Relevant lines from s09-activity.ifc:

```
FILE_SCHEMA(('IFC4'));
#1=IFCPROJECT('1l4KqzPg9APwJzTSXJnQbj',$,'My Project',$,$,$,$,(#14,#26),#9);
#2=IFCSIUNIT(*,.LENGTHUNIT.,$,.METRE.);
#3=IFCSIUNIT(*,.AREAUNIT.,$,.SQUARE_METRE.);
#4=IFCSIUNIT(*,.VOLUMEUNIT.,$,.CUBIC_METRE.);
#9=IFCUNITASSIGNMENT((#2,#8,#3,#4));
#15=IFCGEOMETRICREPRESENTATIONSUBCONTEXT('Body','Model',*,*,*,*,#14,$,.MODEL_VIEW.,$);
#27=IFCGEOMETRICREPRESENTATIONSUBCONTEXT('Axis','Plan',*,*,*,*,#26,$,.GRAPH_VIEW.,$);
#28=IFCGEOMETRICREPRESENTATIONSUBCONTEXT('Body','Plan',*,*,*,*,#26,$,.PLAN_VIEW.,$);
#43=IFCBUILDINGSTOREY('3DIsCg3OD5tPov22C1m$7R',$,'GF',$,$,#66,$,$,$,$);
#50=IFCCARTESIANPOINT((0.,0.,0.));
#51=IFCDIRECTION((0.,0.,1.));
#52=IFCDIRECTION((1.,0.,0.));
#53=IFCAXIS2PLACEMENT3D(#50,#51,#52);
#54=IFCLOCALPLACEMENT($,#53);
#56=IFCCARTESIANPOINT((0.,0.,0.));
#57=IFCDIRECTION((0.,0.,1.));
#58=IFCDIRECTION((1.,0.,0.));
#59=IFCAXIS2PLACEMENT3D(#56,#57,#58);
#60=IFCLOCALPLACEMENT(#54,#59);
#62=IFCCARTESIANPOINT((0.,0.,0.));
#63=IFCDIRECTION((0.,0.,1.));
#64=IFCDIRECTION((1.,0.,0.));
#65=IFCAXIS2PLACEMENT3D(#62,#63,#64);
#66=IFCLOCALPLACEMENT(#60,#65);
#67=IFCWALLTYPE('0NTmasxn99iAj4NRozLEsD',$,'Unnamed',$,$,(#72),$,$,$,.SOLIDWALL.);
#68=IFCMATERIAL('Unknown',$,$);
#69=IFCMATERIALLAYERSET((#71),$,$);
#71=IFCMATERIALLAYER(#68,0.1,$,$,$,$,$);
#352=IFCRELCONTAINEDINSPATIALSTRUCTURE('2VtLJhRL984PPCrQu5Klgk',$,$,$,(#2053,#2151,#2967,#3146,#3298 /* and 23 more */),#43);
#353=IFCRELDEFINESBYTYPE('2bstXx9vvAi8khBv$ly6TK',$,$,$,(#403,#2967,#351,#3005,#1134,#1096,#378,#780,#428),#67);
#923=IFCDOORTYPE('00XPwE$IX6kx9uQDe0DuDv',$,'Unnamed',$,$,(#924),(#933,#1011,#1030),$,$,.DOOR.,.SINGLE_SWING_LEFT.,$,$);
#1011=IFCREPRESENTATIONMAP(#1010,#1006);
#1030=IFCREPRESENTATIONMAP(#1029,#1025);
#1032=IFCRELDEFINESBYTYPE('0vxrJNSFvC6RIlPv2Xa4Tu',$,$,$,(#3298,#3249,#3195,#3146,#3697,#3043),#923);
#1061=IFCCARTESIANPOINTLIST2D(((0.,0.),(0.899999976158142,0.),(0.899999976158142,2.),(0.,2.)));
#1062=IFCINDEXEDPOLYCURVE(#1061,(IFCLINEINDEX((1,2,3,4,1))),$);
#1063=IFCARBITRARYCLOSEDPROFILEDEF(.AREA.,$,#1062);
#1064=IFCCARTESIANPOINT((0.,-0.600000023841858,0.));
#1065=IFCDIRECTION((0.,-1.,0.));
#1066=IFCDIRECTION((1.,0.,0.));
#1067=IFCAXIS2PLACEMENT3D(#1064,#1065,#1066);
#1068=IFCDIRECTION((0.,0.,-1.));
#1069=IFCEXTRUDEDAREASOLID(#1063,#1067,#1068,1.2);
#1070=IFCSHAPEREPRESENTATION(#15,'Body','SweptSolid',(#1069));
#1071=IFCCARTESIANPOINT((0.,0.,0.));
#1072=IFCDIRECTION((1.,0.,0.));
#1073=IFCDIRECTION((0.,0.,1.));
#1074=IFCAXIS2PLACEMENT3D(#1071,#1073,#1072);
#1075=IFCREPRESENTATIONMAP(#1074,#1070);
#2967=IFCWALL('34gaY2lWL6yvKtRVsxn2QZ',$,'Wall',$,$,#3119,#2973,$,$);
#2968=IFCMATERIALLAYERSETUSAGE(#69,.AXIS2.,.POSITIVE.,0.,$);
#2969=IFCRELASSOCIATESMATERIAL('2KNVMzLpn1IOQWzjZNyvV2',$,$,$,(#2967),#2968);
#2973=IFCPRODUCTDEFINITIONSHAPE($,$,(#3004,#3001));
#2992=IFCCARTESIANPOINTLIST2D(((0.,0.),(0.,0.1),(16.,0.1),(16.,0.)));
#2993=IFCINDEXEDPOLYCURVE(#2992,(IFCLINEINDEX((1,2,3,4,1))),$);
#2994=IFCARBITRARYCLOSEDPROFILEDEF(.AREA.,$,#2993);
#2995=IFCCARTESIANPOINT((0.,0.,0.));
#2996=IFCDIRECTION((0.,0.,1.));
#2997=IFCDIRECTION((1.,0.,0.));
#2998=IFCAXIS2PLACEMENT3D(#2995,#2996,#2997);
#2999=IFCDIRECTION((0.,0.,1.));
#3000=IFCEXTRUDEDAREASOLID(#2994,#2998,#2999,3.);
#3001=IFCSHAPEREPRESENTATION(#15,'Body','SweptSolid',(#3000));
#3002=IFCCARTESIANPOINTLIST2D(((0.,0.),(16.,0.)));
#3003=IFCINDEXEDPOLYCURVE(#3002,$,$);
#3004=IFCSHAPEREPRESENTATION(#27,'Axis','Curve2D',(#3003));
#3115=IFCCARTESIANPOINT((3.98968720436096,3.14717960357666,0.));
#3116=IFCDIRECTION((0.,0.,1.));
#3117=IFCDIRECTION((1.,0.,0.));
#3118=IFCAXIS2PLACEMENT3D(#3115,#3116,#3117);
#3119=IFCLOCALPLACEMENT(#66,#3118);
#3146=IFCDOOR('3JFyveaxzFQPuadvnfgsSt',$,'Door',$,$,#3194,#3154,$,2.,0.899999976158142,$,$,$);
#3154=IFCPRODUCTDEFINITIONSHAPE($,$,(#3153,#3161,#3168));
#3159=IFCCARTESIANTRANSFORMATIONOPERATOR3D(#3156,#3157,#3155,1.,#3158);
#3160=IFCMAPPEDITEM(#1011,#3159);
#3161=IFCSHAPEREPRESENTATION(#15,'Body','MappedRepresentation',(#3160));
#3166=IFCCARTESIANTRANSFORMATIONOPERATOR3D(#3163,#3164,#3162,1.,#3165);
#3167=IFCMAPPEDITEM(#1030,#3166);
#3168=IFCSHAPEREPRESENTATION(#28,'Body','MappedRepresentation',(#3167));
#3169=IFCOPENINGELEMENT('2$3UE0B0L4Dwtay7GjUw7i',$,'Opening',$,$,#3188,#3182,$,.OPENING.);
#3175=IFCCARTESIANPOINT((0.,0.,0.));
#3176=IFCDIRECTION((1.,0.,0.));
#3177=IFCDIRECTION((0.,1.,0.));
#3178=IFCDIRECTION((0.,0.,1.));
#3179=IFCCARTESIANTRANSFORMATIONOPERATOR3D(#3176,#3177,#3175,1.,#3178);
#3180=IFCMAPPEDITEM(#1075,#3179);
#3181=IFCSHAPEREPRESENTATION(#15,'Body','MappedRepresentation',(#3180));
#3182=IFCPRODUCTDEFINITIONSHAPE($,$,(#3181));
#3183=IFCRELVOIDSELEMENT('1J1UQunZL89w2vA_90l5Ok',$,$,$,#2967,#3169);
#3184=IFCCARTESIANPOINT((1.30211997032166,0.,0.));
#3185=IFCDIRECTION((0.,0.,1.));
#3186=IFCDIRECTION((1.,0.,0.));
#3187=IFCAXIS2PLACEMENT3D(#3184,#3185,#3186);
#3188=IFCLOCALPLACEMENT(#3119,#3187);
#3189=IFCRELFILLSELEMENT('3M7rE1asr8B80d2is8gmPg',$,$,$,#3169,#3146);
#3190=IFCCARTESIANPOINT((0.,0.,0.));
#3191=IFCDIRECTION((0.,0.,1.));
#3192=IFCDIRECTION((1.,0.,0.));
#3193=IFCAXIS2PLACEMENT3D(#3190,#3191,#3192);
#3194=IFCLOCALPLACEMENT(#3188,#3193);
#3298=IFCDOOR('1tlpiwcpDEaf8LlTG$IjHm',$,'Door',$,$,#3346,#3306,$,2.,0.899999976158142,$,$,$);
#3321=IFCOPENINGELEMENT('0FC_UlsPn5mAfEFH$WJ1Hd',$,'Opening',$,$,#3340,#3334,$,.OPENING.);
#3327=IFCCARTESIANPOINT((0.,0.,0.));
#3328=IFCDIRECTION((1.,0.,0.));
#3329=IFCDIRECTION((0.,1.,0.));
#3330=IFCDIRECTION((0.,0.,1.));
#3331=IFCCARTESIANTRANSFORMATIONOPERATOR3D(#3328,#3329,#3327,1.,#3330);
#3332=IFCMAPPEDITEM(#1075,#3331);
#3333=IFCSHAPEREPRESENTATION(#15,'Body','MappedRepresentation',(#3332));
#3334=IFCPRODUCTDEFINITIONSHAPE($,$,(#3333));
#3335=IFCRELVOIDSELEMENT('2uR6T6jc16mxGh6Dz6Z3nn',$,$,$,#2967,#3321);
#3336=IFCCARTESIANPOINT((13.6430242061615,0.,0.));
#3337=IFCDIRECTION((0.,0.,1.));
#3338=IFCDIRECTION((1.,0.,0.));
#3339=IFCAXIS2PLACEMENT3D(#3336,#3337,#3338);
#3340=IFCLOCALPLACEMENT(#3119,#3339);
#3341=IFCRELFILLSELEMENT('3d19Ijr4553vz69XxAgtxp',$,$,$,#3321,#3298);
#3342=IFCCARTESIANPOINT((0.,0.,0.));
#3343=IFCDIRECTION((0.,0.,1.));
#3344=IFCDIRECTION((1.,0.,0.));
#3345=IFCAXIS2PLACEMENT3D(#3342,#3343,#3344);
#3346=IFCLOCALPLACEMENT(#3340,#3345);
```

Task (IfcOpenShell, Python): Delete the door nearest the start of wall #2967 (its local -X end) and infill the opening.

```python
import ifcopenshell
import ifcopenshell.api.feature
import ifcopenshell.api.root
import ifcopenshell.geom
import ifcopenshell.util.shape

model = ifcopenshell.open("s09-activity.ifc")
settings = ifcopenshell.geom.settings()


def volume(element):
    """Net volume in cubic metres, openings subtracted."""
    shape = ifcopenshell.geom.create_shape(settings, element)
    return ifcopenshell.util.shape.get_volume(shape.geometry)


door = model.by_id(3146)
opening = door.FillsVoids[0].RelatingOpeningElement
wall = opening.VoidsElements[0].RelatingBuildingElement
before = volume(wall)

ifcopenshell.api.root.remove_product(model, product=door)
ifcopenshell.api.feature.remove_feature(model, feature=opening)

after = volume(wall)

print(f"wall volume {before:.3f} -> {after:.3f} m3")

model.write("s09-activity_edited.ifc")
```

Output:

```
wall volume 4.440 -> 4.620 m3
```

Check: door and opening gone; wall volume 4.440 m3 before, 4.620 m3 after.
